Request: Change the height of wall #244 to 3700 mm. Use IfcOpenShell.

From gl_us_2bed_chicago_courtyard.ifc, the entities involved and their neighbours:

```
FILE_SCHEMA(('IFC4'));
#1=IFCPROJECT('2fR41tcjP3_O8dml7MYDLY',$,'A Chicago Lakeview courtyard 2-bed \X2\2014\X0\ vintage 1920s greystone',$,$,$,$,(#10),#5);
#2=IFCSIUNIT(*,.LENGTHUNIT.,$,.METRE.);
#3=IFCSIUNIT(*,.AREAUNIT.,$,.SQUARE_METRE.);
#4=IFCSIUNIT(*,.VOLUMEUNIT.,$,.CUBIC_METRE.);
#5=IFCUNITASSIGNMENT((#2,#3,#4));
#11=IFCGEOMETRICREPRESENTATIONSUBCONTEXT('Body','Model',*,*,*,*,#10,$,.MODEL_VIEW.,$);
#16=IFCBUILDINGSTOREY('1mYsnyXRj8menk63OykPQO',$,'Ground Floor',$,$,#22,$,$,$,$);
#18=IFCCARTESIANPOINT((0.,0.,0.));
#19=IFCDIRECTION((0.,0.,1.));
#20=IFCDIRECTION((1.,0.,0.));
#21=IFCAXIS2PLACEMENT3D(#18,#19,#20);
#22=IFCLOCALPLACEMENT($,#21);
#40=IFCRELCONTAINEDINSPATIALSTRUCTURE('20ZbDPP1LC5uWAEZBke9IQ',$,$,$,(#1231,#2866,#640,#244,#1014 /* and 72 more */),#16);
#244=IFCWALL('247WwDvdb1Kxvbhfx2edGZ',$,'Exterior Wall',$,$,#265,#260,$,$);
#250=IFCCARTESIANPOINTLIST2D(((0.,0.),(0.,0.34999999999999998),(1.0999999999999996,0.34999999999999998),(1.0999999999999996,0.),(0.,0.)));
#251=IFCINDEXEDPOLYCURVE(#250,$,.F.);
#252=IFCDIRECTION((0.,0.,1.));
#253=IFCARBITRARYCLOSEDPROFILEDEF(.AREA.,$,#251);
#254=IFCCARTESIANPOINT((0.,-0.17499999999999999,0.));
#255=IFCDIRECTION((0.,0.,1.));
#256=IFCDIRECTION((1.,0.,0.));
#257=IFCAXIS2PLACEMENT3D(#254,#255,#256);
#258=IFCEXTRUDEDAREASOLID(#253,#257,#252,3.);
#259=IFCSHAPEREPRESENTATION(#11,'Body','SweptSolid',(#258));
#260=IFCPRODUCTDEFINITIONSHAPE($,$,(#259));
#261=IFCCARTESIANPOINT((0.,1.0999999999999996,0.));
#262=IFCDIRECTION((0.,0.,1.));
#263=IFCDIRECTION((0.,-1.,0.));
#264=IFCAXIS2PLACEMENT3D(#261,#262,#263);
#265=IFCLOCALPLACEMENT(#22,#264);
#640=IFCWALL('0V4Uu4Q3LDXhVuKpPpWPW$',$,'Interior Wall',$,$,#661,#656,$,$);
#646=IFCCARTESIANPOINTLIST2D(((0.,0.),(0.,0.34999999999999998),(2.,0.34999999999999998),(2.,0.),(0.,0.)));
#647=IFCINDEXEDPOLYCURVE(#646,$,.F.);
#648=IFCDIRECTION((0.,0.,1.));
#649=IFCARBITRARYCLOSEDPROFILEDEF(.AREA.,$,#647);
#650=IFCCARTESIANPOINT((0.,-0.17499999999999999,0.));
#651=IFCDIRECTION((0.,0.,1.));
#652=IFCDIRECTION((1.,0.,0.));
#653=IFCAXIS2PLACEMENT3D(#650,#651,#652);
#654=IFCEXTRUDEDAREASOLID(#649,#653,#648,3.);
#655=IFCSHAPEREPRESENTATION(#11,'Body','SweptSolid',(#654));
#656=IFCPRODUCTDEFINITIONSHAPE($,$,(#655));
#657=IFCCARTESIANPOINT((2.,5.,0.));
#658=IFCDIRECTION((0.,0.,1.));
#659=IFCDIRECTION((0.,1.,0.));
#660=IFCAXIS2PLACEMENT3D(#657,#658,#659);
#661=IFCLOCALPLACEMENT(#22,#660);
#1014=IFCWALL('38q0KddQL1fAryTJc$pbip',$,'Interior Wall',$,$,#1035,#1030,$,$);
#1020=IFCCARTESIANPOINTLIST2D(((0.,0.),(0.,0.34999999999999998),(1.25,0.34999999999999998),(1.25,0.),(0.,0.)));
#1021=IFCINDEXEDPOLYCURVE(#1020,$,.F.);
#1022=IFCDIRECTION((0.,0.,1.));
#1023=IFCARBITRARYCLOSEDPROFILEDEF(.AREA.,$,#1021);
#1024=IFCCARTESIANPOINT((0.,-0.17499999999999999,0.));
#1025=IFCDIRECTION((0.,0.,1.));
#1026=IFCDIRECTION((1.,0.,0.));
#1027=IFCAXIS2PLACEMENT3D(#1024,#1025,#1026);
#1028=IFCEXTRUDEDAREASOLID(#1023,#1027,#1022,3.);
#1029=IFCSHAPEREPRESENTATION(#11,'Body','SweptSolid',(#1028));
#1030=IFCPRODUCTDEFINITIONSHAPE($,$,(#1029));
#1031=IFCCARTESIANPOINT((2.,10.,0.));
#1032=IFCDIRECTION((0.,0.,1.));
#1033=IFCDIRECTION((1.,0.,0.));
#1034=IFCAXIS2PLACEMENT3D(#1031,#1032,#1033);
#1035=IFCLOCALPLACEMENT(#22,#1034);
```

```python
import ifcopenshell
import ifcopenshell.geom
import ifcopenshell.util.representation
import ifcopenshell.util.shape
import ifcopenshell.util.unit

model = ifcopenshell.open("gl_us_2bed_chicago_courtyard.ifc")
unit_scale = ifcopenshell.util.unit.calculate_unit_scale(model)
settings = ifcopenshell.geom.settings()


def volume(element):
    """Net volume in cubic metres, openings subtracted."""
    shape = ifcopenshell.geom.create_shape(settings, element)
    return ifcopenshell.util.shape.get_volume(shape.geometry)


wall = model.by_guid("247WwDvdb1Kxvbhfx2edGZ")
before = volume(wall)

body = ifcopenshell.util.representation.get_representation(wall, "Model", "Body")
solid = body.Items[0]
old_height = solid.Depth
solid.Depth = 3.7 / unit_scale
after = volume(wall)

print(f"height {old_height:g} -> {solid.Depth:g}, volume {before:.3f} -> {after:.3f} m3")

model.write("gl_us_2bed_chicago_courtyard_rev.ifc")
```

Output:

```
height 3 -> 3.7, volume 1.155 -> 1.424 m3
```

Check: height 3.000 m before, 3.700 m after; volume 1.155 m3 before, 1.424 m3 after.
